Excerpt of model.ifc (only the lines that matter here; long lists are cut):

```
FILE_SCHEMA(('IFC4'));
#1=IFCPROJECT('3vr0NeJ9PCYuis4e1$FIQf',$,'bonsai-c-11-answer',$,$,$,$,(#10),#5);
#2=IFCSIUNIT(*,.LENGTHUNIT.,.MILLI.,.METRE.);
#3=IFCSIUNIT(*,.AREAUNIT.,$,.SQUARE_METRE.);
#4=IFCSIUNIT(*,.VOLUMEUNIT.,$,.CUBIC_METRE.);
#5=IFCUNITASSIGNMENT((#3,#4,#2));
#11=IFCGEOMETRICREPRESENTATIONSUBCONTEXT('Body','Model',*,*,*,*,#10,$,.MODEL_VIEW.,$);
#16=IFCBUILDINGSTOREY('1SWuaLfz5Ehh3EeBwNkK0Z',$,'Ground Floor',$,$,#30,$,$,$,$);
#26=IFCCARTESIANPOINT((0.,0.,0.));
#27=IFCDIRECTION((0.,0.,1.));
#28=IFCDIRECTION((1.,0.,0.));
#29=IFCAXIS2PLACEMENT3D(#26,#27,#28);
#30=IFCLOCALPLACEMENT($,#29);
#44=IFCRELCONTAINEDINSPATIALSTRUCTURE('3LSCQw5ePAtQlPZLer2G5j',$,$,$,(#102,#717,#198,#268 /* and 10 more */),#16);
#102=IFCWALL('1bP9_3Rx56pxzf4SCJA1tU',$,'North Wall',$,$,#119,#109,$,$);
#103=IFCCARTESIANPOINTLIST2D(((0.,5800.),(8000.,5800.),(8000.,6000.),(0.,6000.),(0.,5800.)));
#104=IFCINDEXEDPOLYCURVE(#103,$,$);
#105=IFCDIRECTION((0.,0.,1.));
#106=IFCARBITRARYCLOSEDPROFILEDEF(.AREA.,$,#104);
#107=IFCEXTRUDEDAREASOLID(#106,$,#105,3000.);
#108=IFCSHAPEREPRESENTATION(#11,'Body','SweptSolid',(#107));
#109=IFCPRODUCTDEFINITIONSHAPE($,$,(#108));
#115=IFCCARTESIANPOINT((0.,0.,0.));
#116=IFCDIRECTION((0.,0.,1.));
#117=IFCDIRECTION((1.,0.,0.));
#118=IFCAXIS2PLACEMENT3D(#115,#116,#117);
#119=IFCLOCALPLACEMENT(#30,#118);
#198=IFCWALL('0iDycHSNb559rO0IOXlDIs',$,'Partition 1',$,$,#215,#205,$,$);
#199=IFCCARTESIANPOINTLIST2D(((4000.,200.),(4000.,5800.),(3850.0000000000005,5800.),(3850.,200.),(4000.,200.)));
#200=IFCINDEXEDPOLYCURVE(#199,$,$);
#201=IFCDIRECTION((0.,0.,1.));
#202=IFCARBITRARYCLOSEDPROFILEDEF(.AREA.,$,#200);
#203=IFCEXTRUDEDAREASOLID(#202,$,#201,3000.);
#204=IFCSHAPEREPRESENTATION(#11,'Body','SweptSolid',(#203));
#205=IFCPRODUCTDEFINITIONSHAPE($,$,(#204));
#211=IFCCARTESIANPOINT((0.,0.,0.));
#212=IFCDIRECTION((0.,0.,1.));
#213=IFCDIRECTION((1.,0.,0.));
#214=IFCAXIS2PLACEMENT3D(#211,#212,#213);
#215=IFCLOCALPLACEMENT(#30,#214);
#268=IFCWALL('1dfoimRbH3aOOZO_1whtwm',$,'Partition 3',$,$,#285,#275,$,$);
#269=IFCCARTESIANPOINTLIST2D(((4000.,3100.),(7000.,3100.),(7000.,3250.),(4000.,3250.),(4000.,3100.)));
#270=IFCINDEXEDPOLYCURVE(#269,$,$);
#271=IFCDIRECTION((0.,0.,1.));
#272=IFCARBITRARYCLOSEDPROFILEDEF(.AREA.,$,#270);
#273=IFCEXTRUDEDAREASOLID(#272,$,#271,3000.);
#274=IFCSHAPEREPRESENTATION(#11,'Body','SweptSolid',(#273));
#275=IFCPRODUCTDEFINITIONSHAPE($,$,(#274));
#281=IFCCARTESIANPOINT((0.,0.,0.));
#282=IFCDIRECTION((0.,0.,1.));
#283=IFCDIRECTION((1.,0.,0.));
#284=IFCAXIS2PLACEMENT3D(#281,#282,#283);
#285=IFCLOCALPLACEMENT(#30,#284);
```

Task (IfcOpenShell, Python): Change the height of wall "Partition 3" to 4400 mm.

```python
import ifcopenshell
import ifcopenshell.geom
import ifcopenshell.util.representation
import ifcopenshell.util.shape

model = ifcopenshell.open("model.ifc")
settings = ifcopenshell.geom.settings()


def volume(element):
    """Net volume in cubic metres, openings subtracted."""
    shape = ifcopenshell.geom.create_shape(settings, element)
    return ifcopenshell.util.shape.get_volume(shape.geometry)


wall = model.by_id(268)
before = volume(wall)

body = ifcopenshell.util.representation.get_representation(wall, "Model", "Body")
solid = body.Items[0]
old_height = solid.Depth
solid.Depth = 4400.0
after = volume(wall)

print(f"height {old_height:g} -> {solid.Depth:g}, volume {before:.3f} -> {after:.3f} m3")

model.write("model_updated.ifc")
```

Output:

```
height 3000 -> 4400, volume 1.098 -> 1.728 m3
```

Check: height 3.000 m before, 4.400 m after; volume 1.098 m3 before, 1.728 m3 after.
